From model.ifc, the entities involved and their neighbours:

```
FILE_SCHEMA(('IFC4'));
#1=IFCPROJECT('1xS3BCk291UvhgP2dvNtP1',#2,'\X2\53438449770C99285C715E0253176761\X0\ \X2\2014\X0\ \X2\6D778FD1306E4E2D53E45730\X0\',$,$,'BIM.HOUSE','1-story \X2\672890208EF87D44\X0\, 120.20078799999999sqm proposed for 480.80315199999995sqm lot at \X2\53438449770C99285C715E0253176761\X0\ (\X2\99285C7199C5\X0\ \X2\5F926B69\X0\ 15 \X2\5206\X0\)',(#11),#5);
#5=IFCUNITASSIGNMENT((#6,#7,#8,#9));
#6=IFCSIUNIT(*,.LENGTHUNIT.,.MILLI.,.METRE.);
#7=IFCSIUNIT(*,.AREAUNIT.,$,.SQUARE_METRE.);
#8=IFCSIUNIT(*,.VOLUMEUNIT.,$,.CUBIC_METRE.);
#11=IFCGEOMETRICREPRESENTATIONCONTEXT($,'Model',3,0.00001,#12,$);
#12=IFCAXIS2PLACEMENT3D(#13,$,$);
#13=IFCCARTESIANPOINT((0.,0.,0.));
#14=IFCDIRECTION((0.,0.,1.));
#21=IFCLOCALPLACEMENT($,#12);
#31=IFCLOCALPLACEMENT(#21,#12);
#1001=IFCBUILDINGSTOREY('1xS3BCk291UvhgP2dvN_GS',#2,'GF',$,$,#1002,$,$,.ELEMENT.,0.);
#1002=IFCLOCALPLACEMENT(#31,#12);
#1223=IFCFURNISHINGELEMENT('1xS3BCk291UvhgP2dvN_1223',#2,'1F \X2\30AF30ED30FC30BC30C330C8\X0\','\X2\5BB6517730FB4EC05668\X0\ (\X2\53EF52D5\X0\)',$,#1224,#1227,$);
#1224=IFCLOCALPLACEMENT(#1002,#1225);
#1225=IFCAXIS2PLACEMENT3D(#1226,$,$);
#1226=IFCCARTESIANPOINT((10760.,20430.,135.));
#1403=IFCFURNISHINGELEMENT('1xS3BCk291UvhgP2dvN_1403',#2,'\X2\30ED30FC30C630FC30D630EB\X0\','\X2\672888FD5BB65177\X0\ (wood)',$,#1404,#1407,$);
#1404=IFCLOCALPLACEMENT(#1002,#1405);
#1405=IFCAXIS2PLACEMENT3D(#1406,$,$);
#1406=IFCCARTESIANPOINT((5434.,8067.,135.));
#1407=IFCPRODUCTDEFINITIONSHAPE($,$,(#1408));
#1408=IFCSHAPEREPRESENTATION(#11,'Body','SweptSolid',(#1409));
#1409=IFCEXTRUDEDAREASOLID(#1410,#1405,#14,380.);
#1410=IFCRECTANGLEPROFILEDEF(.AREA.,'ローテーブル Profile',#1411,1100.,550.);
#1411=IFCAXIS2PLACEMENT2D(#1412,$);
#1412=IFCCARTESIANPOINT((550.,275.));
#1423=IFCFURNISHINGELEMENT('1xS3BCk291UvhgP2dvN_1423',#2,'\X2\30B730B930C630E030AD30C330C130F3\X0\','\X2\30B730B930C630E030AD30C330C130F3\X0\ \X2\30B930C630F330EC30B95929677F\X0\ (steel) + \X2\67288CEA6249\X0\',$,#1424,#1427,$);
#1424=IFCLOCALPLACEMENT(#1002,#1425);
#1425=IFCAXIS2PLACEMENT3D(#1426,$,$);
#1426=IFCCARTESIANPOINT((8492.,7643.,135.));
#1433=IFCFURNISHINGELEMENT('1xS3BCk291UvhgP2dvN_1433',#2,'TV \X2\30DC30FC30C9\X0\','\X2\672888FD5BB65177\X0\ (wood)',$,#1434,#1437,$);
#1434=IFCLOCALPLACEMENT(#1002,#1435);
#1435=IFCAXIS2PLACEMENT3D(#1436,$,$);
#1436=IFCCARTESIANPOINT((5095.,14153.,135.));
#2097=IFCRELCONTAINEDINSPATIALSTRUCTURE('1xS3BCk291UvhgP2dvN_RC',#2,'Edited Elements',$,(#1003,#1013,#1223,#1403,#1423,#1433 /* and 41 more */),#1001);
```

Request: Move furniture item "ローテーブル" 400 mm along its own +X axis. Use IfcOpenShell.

```python
import ifcopenshell
import ifcopenshell.api.geometry
import ifcopenshell.util.placement

model = ifcopenshell.open("model.ifc")

item = model.by_guid("1xS3BCk291UvhgP2dvN_1403")
matrix = ifcopenshell.util.placement.get_local_placement(item.ObjectPlacement)
matrix[:3, 3] += matrix[:3, 0] * 400.0
ifcopenshell.api.geometry.edit_object_placement(model, product=item, matrix=matrix, is_si=False)

print(ifcopenshell.util.placement.get_local_placement(item.ObjectPlacement).round(3) + 0.0)

model.write("model-out.ifc")
```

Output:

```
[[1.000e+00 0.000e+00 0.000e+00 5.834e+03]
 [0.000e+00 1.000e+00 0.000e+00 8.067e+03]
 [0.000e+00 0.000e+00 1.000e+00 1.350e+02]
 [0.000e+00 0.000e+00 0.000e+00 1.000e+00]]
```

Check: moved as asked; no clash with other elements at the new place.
